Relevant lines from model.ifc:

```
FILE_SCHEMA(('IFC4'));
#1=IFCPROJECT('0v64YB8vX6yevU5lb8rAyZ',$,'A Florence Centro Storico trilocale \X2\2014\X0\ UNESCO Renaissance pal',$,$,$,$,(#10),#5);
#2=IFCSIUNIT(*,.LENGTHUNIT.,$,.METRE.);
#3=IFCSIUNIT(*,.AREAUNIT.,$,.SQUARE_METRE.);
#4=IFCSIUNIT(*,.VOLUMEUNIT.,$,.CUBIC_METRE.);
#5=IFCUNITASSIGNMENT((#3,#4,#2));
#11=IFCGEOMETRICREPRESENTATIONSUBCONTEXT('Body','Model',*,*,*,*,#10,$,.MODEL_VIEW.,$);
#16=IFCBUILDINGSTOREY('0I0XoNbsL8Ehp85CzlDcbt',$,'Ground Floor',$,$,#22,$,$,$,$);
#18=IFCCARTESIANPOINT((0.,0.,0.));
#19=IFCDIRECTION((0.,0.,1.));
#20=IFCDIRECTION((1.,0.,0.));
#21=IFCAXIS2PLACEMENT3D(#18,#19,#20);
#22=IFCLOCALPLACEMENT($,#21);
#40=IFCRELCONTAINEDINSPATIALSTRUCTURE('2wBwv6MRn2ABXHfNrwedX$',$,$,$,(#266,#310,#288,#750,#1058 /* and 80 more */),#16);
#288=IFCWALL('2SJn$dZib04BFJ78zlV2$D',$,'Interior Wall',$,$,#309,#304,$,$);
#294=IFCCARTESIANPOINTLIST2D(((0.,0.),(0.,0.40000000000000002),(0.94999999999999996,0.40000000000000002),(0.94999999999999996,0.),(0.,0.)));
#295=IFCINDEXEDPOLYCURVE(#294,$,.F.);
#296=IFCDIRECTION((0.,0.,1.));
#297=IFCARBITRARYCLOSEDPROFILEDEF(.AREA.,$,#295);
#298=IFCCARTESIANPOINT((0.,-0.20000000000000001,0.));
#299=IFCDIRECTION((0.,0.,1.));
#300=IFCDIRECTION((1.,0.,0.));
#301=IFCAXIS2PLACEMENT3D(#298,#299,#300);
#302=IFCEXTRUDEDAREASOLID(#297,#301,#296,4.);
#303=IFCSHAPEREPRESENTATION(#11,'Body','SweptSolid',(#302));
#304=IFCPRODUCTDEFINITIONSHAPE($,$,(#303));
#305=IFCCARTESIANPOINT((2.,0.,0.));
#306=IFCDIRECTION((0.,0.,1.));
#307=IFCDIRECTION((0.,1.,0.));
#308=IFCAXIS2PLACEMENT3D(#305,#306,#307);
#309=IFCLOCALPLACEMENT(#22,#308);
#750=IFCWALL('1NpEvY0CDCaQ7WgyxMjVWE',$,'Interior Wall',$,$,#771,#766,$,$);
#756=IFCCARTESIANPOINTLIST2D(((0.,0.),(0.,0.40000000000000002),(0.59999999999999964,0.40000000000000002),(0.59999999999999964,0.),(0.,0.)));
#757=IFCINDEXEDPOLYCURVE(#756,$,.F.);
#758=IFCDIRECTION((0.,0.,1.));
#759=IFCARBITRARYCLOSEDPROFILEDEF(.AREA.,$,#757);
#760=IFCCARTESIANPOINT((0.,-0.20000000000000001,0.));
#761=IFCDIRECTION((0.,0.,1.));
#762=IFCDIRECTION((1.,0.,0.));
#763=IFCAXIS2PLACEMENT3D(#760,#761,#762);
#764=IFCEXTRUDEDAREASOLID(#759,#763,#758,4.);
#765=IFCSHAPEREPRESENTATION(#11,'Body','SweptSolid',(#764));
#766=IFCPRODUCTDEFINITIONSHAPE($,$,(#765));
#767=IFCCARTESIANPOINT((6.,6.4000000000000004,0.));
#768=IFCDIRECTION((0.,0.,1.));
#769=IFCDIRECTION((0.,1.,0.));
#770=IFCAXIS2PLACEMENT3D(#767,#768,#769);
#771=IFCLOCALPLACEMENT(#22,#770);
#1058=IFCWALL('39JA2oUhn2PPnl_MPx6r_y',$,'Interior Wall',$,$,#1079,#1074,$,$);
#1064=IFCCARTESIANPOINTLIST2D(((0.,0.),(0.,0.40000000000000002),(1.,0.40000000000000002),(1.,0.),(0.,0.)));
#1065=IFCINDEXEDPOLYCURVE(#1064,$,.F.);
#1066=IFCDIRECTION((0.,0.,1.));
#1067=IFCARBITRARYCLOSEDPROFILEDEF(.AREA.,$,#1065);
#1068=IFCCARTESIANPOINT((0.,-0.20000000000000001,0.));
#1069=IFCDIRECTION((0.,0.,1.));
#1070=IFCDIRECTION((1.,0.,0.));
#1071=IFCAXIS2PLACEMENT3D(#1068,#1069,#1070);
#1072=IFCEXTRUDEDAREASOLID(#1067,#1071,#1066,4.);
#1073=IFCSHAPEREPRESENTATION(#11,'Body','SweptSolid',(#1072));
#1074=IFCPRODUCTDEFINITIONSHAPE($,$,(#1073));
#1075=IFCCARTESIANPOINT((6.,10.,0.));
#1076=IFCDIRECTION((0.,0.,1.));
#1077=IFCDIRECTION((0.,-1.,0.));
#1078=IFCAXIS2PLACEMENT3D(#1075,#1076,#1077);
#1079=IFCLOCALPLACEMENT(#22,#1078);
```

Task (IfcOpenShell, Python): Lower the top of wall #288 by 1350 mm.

```python
import ifcopenshell
import ifcopenshell.geom
import ifcopenshell.util.representation
import ifcopenshell.util.shape
import ifcopenshell.util.unit

model = ifcopenshell.open("model.ifc")
unit_scale = ifcopenshell.util.unit.calculate_unit_scale(model)
settings = ifcopenshell.geom.settings()


def volume(element):
    """Net volume in cubic metres, openings subtracted."""
    shape = ifcopenshell.geom.create_shape(settings, element)
    return ifcopenshell.util.shape.get_volume(shape.geometry)


wall = model.by_guid("2SJn$dZib04BFJ78zlV2$D")
before = volume(wall)

body = ifcopenshell.util.representation.get_representation(wall, "Model", "Body")
solid = body.Items[0]
old_height = solid.Depth
solid.Depth -= 1.35 / unit_scale
after = volume(wall)

print(f"height {old_height:g} -> {solid.Depth:g}, volume {before:.3f} -> {after:.3f} m3")

model.write("model-out.ifc")
```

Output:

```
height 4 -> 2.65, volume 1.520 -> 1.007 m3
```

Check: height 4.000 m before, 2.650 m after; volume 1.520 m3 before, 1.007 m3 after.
